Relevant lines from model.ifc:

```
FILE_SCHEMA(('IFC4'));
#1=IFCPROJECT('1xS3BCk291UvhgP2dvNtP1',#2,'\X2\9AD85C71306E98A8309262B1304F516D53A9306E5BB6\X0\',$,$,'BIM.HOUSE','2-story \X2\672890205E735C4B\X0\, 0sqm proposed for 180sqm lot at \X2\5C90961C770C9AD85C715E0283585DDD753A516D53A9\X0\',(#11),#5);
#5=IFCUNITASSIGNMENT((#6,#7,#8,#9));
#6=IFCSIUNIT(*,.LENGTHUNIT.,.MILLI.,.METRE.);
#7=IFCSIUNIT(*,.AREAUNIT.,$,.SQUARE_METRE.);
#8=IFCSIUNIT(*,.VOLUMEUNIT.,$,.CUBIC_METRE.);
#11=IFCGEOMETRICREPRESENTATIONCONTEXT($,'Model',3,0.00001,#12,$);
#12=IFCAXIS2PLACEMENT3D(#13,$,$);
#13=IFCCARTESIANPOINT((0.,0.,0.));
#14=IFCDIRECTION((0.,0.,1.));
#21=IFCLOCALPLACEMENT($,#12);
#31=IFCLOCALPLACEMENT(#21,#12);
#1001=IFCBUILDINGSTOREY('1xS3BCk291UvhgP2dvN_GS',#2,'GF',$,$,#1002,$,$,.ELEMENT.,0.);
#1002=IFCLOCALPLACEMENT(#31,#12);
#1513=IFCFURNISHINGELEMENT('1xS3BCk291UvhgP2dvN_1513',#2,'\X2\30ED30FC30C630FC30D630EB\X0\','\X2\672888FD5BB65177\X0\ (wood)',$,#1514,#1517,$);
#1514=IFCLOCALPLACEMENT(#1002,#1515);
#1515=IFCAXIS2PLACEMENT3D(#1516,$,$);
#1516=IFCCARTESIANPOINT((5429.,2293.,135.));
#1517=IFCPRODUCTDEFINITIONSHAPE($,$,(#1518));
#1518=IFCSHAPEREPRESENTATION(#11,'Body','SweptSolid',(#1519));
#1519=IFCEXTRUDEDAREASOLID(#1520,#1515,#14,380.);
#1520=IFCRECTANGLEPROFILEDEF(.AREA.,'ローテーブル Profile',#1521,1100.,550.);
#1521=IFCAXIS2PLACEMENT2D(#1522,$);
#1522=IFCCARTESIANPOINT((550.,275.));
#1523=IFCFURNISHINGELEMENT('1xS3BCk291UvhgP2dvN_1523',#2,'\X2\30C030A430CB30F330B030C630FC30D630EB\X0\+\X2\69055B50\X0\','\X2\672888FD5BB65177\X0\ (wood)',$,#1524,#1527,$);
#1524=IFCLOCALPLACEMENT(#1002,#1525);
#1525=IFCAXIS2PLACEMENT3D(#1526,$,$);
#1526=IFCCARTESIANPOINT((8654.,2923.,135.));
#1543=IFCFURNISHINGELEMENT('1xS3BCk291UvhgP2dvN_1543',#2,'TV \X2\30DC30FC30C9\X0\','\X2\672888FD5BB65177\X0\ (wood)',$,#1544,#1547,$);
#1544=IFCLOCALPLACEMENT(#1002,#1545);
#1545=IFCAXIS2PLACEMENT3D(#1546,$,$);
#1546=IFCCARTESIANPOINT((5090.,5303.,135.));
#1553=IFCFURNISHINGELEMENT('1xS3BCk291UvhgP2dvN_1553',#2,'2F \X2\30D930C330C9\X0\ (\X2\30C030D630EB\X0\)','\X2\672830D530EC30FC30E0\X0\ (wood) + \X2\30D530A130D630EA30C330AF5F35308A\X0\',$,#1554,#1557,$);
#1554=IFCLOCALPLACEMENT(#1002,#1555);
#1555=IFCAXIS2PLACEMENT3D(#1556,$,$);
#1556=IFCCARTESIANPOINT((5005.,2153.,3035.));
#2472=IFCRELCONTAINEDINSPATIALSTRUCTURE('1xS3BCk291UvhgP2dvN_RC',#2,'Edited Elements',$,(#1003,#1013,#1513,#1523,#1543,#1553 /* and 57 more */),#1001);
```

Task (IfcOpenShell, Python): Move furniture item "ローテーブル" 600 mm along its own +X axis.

```python
import ifcopenshell
import ifcopenshell.api.geometry
import ifcopenshell.util.placement
import ifcopenshell.util.unit

model = ifcopenshell.open("model.ifc")
unit_scale = ifcopenshell.util.unit.calculate_unit_scale(model)

item = model.by_id(1513)
matrix = ifcopenshell.util.placement.get_local_placement(item.ObjectPlacement)
matrix[:3, 3] += matrix[:3, 0] * 0.6 / unit_scale
ifcopenshell.api.geometry.edit_object_placement(model, product=item, matrix=matrix, is_si=False)

print(ifcopenshell.util.placement.get_local_placement(item.ObjectPlacement).round(3) + 0.0)

model.write("model_updated.ifc")
```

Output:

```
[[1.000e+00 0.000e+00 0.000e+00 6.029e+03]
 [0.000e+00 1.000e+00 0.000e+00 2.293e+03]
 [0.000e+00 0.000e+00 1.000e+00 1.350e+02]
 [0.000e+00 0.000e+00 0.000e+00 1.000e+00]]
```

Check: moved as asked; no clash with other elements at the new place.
